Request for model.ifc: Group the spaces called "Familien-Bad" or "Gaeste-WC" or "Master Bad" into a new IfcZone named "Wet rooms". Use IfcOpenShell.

First a look at what the model holds.

```python
import ifcopenshell

model = ifcopenshell.open("model.ifc")
print(model.schema)
seen = {}
for space in model.by_type("IfcSpace"):
    seen[space.LongName] = seen.get(space.LongName, 0) + 1
for name, count in sorted(seen.items(), key=str):
    print(count, "x", name)
print("zones:", [z.Name for z in model.by_type("IfcZone")][:20])
```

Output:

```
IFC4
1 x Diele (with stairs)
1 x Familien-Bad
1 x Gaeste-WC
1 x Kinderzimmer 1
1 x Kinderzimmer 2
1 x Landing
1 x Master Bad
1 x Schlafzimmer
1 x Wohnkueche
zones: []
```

```python
import ifcopenshell
import ifcopenshell.api.group
import ifcopenshell.api.root

model = ifcopenshell.open("model.ifc")

names = {"Familien-Bad", "Gaeste-WC", "Master Bad"}
spaces = [s for s in model.by_type("IfcSpace") if s.LongName in names]

zone = ifcopenshell.api.root.create_entity(model, ifc_class="IfcZone", name="Wet rooms")
ifcopenshell.api.group.assign_group(model, products=spaces, group=zone)
print(len(spaces), "spaces in", zone.Name)

model.write("model_edited.ifc")
```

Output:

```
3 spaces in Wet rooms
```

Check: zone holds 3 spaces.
